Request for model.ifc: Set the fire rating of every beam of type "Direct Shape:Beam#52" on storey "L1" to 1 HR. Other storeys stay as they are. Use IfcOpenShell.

First a look at what the model holds.

```python
import ifcopenshell
import ifcopenshell.util.element

model = ifcopenshell.open("model.ifc")
print(model.schema)
storey = next(s for s in model.by_type("IfcBuildingStorey") if s.Name == "L1")
beams = [e for e in ifcopenshell.util.element.get_decomposition(storey) if e.is_a("IfcBeam")]
seen = {}
for e in beams:
    element_type = ifcopenshell.util.element.get_type(e)
    key = (element_type.Name if element_type != e and element_type else None, ifcopenshell.util.element.get_pset(e, "Pset_BeamCommon", "FireRating"))
    seen[key] = seen.get(key, 0) + 1
for (name, value), count in sorted(seen.items(), key=str):
    print(count, "x", name, "|", value)
```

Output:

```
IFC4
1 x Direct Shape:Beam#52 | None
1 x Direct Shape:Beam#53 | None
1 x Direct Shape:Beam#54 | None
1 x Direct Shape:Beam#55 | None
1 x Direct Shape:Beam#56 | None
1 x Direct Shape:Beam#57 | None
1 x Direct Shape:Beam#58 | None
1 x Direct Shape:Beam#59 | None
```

```python
import ifcopenshell
import ifcopenshell.api.pset
import ifcopenshell.util.element

model = ifcopenshell.open("model.ifc")

storey = next(s for s in model.by_type("IfcBuildingStorey") if s.Name == "L1")
beams = [e for e in ifcopenshell.util.element.get_decomposition(storey) if e.is_a("IfcBeam")]

count = 0
for e in beams:
    element_type = ifcopenshell.util.element.get_type(e)
    if element_type in (None, e) or element_type.Name != "Direct Shape:Beam#52":
        continue
    # add_pset returns the element's existing set when there is one.
    pset = ifcopenshell.api.pset.add_pset(model, product=e, name="Pset_BeamCommon")
    ifcopenshell.api.pset.edit_pset(model, pset=pset, properties={"FireRating": "1 HR"})
    count += 1

print(count, "beams updated")

model.write("model_rev.ifc")
```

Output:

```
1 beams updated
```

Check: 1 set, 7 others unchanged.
